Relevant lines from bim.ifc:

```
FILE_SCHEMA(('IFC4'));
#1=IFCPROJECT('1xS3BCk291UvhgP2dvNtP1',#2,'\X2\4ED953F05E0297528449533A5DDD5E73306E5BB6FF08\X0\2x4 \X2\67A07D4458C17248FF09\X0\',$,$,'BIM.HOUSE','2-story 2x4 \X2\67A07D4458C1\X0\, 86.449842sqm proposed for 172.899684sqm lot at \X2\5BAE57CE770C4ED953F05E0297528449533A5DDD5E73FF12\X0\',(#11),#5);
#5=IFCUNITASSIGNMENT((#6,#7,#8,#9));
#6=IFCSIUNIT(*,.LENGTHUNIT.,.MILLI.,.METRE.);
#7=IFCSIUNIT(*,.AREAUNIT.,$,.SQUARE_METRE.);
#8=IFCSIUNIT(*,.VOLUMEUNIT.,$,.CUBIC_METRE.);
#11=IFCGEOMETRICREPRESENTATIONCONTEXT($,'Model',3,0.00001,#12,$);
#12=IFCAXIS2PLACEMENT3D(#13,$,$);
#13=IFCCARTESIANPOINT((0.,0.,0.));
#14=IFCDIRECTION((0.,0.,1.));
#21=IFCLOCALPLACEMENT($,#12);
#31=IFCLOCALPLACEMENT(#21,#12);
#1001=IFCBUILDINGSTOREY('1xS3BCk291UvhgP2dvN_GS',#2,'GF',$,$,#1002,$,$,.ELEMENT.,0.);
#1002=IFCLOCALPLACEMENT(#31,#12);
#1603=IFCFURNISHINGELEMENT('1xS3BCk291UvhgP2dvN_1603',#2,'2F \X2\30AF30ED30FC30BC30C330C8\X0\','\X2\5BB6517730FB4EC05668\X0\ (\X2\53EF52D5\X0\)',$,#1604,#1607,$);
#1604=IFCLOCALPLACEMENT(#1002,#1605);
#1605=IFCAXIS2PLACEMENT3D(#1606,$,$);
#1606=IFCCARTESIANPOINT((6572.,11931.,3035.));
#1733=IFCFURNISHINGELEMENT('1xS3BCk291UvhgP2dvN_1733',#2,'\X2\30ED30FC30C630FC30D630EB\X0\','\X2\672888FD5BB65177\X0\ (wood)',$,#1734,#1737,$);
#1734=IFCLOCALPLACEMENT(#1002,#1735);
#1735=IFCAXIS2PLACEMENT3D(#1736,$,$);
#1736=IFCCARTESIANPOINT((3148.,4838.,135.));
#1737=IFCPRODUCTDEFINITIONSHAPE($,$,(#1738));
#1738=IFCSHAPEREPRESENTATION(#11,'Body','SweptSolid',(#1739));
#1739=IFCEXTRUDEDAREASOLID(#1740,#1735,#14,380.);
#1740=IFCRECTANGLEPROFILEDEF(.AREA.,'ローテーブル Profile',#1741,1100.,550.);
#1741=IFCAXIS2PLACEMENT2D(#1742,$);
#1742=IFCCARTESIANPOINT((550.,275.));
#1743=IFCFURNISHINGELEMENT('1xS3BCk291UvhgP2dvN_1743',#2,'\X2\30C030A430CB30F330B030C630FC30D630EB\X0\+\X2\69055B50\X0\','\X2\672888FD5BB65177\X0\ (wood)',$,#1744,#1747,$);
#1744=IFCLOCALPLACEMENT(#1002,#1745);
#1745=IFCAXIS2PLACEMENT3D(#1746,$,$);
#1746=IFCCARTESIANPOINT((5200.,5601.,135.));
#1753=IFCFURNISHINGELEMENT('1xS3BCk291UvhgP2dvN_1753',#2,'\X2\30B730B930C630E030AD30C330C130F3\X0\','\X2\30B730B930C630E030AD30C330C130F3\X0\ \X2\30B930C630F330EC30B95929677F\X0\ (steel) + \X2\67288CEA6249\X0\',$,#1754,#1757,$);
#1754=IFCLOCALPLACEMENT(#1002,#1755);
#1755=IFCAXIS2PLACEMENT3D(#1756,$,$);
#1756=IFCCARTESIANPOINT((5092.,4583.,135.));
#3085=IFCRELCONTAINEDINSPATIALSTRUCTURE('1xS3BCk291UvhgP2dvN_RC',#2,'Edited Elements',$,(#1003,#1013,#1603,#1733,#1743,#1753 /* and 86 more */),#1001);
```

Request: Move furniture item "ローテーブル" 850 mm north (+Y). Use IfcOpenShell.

```python
import ifcopenshell
import ifcopenshell.api.geometry
import ifcopenshell.util.placement
import ifcopenshell.util.unit

model = ifcopenshell.open("bim.ifc")
unit_scale = ifcopenshell.util.unit.calculate_unit_scale(model)

item = model.by_guid("1xS3BCk291UvhgP2dvN_1733")
matrix = ifcopenshell.util.placement.get_local_placement(item.ObjectPlacement)
matrix[1, 3] += 0.85 / unit_scale
ifcopenshell.api.geometry.edit_object_placement(model, product=item, matrix=matrix, is_si=False)

print(ifcopenshell.util.placement.get_local_placement(item.ObjectPlacement).round(3) + 0.0)

model.write("bim_rev.ifc")
```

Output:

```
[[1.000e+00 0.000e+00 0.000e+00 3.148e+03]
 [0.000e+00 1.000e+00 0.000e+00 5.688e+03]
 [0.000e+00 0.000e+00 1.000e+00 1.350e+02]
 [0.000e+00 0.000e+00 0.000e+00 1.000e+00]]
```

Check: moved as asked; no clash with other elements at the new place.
